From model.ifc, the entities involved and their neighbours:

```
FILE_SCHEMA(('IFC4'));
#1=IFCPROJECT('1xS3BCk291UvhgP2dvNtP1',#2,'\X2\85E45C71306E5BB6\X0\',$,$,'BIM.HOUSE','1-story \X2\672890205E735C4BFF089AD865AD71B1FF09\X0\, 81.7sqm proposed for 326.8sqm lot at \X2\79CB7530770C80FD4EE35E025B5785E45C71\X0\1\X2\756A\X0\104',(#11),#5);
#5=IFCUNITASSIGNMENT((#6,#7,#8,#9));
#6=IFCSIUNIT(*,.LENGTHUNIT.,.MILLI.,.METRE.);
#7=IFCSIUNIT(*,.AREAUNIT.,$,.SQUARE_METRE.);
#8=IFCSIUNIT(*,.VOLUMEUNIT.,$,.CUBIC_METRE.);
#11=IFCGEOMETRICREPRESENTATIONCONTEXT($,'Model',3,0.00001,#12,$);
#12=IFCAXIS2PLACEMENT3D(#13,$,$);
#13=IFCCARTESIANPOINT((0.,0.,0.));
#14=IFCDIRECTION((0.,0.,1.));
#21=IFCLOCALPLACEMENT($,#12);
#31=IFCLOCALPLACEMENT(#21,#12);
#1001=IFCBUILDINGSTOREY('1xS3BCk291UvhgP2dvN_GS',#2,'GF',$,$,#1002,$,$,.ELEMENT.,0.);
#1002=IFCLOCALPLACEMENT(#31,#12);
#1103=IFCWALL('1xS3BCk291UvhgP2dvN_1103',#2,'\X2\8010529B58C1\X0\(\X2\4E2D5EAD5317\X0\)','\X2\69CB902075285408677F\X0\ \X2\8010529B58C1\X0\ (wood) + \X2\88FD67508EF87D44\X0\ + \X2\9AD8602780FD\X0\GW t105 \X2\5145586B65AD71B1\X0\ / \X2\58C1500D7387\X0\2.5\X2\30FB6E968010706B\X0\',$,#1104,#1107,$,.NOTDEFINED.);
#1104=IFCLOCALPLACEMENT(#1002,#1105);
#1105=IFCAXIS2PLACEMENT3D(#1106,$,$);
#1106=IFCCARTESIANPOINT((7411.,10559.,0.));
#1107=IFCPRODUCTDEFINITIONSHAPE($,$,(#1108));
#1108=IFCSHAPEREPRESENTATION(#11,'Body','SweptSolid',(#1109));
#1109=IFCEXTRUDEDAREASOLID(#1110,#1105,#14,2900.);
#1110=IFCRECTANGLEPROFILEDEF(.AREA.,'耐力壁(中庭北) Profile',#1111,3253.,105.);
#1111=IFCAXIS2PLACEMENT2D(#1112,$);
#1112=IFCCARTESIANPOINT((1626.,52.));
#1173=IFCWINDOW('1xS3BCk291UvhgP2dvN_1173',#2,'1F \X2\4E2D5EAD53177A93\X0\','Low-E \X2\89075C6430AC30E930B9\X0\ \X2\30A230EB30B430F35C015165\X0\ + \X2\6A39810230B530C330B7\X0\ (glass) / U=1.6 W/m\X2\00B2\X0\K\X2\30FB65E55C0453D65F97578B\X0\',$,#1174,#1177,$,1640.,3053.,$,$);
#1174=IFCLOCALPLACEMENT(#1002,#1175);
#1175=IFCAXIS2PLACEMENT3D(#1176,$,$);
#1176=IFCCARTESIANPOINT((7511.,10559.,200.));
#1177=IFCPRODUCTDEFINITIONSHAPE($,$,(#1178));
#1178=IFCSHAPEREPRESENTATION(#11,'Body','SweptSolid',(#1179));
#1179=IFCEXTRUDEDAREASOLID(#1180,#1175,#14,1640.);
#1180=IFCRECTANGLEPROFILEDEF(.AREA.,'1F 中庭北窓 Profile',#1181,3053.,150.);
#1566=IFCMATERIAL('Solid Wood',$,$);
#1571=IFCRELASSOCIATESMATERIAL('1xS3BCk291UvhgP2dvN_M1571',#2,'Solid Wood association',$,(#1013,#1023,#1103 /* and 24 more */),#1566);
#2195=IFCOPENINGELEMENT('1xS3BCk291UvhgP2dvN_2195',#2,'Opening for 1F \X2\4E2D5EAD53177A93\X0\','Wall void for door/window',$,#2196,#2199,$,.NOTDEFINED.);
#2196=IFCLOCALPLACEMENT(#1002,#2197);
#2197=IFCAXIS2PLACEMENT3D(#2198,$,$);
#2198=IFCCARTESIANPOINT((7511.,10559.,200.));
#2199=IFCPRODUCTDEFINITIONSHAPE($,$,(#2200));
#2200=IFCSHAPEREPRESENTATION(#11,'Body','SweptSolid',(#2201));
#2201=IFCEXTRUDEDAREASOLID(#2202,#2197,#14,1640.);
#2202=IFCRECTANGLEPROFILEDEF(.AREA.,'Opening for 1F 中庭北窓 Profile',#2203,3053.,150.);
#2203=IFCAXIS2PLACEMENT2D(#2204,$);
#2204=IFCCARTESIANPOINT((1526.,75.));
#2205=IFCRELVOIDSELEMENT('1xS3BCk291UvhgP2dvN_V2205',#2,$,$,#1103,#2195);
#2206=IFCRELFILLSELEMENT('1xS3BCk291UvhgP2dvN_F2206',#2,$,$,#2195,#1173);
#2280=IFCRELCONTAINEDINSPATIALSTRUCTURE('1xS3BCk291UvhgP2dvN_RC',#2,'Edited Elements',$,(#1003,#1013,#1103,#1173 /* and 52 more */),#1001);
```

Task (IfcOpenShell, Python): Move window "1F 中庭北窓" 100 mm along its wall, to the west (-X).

```python
import ifcopenshell
import ifcopenshell.api.geometry
import ifcopenshell.util.placement

model = ifcopenshell.open("model.ifc")

window = model.by_guid("1xS3BCk291UvhgP2dvN_1173")
opening = window.FillsVoids[0].RelatingOpeningElement
wall = opening.VoidsElements[0].RelatingBuildingElement

wall_matrix = ifcopenshell.util.placement.get_local_placement(wall.ObjectPlacement)
shift = wall_matrix[:3, 0] * -100.0
before = ifcopenshell.util.placement.get_local_placement(window.ObjectPlacement)[:3, 3].copy()

# The window is not placed relative to its opening, so move both.
for product in (opening, window):
    matrix = ifcopenshell.util.placement.get_local_placement(product.ObjectPlacement)
    matrix[:3, 3] += shift
    ifcopenshell.api.geometry.edit_object_placement(model, product=product, matrix=matrix, is_si=False)

after = ifcopenshell.util.placement.get_local_placement(window.ObjectPlacement)[:3, 3]
print("window moved by", (after - before).round(3) + 0.0)

model.write("model_updated.ifc")
```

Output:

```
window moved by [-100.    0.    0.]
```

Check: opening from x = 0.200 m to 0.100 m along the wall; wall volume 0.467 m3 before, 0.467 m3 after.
